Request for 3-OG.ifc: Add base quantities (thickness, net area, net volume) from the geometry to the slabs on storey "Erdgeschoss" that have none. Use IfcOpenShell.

First a look at what the model holds.

```python
import ifcopenshell
import ifcopenshell.util.element
import ifcopenshell.util.unit

model = ifcopenshell.open("3-OG.ifc")
print(model.schema)
for unit_type in ("LENGTHUNIT", "AREAUNIT", "VOLUMEUNIT"):
    print(unit_type, ifcopenshell.util.unit.calculate_unit_scale(model, unit_type))
storey = next(s for s in model.by_type("IfcBuildingStorey") if s.Name == "Erdgeschoss")
slabs = [e for e in ifcopenshell.util.element.get_decomposition(storey) if e.is_a("IfcSlab")]
for e in sorted(slabs, key=lambda e: e.id()):
    print(e.id(), e.is_a(), e.Name, list(ifcopenshell.util.element.get_psets(e, qtos_only=True)), sep=" | ")
```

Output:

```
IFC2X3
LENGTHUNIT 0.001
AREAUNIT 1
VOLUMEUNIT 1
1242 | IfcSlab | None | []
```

```python
import ifcopenshell
import ifcopenshell.api.pset
import ifcopenshell.geom
import ifcopenshell.util.element
import ifcopenshell.util.shape
import ifcopenshell.util.unit

model = ifcopenshell.open("3-OG.ifc")
unit_scale = ifcopenshell.util.unit.calculate_unit_scale(model)
area_scale = ifcopenshell.util.unit.calculate_unit_scale(model, "AREAUNIT")
volume_scale = ifcopenshell.util.unit.calculate_unit_scale(model, "VOLUMEUNIT")
settings = ifcopenshell.geom.settings()

storey = next(s for s in model.by_type("IfcBuildingStorey") if s.Name == "Erdgeschoss")
slabs = [e for e in ifcopenshell.util.element.get_decomposition(storey) if e.is_a("IfcSlab")]

for e in sorted(slabs, key=lambda e: e.id()):
    if ifcopenshell.util.element.get_psets(e, qtos_only=True, should_inherit=False):
        continue
    # Geometry comes back in metres, in the element's own axes.
    shape = ifcopenshell.geom.create_shape(settings, e)
    values = {
        "Width": ifcopenshell.util.shape.get_z(shape.geometry) / unit_scale,
        "NetArea": ifcopenshell.util.shape.get_footprint_area(shape.geometry) / area_scale,
        "NetVolume": ifcopenshell.util.shape.get_volume(shape.geometry) / volume_scale,
    }
    qto = ifcopenshell.api.pset.add_qto(model, product=e, name="BaseQuantities")
    ifcopenshell.api.pset.edit_qto(model, qto=qto, properties=values)
    print(e.id(), {k: round(v, 3) for k, v in values.items()})

model.write("3-OG_rev.ifc")
```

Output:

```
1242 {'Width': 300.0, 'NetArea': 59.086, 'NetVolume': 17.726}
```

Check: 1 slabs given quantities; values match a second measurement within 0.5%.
